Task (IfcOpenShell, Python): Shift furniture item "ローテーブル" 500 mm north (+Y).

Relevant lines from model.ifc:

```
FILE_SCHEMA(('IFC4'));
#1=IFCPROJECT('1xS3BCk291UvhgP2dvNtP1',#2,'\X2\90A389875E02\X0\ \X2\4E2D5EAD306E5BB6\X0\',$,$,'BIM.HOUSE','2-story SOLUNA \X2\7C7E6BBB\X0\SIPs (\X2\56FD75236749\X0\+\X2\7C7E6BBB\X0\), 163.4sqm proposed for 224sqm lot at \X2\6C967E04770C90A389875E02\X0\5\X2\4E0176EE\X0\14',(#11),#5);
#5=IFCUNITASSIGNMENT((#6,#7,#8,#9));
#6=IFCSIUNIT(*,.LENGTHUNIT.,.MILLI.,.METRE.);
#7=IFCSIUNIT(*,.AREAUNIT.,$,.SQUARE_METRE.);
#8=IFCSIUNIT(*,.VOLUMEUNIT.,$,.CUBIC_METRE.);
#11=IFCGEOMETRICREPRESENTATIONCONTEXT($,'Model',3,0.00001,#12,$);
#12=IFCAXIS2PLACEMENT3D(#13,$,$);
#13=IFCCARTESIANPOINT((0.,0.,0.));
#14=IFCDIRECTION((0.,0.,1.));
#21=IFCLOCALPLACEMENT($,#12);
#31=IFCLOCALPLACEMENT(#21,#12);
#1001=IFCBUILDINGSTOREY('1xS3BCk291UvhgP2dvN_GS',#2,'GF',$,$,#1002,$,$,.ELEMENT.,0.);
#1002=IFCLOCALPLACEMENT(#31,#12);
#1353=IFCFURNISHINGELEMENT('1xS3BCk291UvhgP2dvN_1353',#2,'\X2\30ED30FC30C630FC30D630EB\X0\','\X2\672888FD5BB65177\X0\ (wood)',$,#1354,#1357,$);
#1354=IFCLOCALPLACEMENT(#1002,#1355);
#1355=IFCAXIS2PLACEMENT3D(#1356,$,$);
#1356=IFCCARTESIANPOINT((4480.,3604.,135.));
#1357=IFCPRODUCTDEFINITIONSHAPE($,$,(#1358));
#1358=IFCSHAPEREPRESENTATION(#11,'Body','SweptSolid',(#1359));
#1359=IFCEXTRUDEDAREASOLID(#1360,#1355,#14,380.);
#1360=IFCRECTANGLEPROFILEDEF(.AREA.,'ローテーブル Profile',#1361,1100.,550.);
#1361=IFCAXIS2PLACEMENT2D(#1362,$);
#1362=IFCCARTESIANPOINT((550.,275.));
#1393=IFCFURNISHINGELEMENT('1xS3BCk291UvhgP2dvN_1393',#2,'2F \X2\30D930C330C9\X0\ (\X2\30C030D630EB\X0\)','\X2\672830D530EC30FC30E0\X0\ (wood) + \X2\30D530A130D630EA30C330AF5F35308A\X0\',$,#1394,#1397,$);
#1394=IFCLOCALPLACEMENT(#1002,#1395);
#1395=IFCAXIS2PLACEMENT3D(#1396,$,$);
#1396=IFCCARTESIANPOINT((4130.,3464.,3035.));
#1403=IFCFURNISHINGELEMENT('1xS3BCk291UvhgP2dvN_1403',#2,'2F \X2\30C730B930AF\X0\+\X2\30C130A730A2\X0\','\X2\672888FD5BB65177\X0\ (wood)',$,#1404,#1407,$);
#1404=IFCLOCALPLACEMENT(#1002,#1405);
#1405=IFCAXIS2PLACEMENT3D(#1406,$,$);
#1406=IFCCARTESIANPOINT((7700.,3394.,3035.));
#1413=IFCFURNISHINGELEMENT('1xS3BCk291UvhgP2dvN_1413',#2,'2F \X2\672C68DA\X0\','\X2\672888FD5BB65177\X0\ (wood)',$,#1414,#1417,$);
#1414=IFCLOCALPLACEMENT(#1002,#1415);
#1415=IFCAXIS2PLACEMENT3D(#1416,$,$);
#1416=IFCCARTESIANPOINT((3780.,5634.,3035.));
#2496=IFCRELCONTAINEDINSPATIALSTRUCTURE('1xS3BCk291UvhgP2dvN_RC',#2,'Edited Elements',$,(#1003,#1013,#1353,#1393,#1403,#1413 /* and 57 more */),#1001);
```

```python
import ifcopenshell
import ifcopenshell.api.geometry
import ifcopenshell.util.placement

model = ifcopenshell.open("model.ifc")

item = model.by_guid("1xS3BCk291UvhgP2dvN_1353")
matrix = ifcopenshell.util.placement.get_local_placement(item.ObjectPlacement)
matrix[1, 3] += 500.0
ifcopenshell.api.geometry.edit_object_placement(model, product=item, matrix=matrix, is_si=False)

print(ifcopenshell.util.placement.get_local_placement(item.ObjectPlacement).round(3) + 0.0)

model.write("model_updated.ifc")
```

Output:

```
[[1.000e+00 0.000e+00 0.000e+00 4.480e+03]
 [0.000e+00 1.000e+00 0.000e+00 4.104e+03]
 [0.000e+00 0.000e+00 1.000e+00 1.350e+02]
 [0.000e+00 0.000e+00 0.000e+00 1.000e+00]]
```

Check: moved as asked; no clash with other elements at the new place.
